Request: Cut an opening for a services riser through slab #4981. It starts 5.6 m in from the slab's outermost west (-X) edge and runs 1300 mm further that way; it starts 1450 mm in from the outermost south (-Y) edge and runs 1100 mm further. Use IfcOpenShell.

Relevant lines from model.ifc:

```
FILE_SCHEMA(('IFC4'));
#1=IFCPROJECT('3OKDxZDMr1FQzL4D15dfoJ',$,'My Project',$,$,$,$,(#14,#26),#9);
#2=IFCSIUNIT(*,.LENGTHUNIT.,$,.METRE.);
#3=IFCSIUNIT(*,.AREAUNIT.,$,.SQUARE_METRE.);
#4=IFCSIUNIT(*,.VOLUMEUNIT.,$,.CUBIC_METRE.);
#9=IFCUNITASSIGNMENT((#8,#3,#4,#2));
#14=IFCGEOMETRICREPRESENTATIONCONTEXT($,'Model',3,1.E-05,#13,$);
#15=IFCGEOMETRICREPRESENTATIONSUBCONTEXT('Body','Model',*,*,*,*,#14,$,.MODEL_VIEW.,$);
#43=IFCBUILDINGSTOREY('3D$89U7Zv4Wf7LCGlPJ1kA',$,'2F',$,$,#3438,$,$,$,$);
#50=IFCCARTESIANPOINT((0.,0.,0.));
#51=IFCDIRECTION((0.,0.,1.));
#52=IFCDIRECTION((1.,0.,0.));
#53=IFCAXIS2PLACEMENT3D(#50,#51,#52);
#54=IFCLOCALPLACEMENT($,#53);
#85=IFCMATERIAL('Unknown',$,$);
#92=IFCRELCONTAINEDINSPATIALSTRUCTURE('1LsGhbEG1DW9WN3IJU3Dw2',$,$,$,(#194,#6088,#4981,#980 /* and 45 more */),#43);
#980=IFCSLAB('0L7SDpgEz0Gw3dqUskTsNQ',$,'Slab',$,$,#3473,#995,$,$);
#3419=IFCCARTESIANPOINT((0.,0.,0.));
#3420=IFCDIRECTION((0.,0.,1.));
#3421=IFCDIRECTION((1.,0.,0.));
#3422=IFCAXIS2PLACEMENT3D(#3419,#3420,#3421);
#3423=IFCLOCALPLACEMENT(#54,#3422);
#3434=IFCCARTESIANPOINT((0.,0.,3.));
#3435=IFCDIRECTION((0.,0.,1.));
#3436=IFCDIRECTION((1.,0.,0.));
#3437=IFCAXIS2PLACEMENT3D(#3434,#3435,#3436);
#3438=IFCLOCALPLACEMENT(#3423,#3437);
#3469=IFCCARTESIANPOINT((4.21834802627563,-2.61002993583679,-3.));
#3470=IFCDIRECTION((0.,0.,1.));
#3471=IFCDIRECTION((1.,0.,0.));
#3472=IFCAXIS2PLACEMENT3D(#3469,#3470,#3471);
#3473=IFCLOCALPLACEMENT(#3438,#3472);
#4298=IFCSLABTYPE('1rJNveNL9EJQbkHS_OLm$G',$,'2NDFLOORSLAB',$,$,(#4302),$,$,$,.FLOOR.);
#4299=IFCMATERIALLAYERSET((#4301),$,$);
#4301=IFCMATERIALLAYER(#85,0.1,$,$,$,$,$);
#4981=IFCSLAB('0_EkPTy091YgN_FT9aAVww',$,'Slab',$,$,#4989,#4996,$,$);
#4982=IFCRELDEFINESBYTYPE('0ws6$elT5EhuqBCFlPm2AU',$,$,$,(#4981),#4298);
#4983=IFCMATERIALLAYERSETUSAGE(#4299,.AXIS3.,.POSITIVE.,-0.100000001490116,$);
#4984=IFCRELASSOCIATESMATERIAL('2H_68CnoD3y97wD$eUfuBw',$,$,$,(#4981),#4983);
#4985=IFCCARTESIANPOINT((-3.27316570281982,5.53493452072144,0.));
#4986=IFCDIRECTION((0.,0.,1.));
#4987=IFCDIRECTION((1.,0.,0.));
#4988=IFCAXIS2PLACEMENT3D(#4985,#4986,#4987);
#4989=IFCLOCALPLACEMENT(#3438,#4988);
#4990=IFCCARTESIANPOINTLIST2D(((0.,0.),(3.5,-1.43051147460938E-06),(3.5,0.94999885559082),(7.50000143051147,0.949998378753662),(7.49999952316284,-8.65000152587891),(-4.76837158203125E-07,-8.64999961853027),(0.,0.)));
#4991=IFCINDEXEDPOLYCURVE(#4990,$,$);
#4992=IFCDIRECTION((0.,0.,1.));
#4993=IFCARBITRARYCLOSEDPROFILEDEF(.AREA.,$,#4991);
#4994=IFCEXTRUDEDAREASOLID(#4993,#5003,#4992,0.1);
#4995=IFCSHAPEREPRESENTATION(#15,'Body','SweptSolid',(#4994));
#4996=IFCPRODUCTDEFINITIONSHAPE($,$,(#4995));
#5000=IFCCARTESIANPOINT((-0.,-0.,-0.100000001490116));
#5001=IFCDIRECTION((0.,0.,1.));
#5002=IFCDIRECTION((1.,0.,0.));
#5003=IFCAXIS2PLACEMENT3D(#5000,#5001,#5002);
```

```python
import numpy as np
import ifcopenshell
import ifcopenshell.api.feature
import ifcopenshell.api.geometry
import ifcopenshell.api.root
import ifcopenshell.geom
import ifcopenshell.util.placement
import ifcopenshell.util.representation
import ifcopenshell.util.shape
import ifcopenshell.util.unit

model = ifcopenshell.open("model.ifc")
unit_scale = ifcopenshell.util.unit.calculate_unit_scale(model)
settings = ifcopenshell.geom.settings()


def volume(element):
    """Net volume in cubic metres, openings subtracted."""
    shape = ifcopenshell.geom.create_shape(settings, element)
    return ifcopenshell.util.shape.get_volume(shape.geometry)


slab = model.by_id(4981)
before = volume(slab)

# Extent in the slab's own axes, in metres. The edges named are its -X and -Y sides.
slab_shape = ifcopenshell.geom.create_shape(settings, slab)
vertices = ifcopenshell.util.shape.get_vertices(slab_shape.geometry)
x_min, y_min, bottom = vertices.min(axis=0)
top = vertices[:, 2].max()

opening = ifcopenshell.api.root.create_entity(model, ifc_class="IfcOpeningElement", name="Services riser opening", predefined_type="OPENING")
context = ifcopenshell.util.representation.get_context(model, "Model", "Body", "MODEL_VIEW")
width, depth = 1.3, 1.1
outline = [(0.0, 0.0), (width, 0.0), (width, depth), (0.0, depth), (0.0, 0.0)]
# Overshoot both faces by 50 mm so the cut is clean.
shape = ifcopenshell.api.geometry.add_slab_representation(
    model, context=context, depth=top - bottom + 0.1, polyline=outline
)
ifcopenshell.api.geometry.assign_representation(model, product=opening, representation=shape)

matrix = ifcopenshell.util.placement.get_local_placement(slab.ObjectPlacement)
matrix[:, 3] = matrix @ np.append(np.array([x_min + 5.6, y_min + 1.45, bottom - 0.05]) / unit_scale, 1.0)
ifcopenshell.api.geometry.edit_object_placement(model, product=opening, matrix=matrix, is_si=False)
ifcopenshell.api.feature.add_feature(model, feature=opening, element=slab)

after = volume(slab)

print(f"slab volume {before:.3f} -> {after:.3f} m3")

model.write("model_v2.ifc")
```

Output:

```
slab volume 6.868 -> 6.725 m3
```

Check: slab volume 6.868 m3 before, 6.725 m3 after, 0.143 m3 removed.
